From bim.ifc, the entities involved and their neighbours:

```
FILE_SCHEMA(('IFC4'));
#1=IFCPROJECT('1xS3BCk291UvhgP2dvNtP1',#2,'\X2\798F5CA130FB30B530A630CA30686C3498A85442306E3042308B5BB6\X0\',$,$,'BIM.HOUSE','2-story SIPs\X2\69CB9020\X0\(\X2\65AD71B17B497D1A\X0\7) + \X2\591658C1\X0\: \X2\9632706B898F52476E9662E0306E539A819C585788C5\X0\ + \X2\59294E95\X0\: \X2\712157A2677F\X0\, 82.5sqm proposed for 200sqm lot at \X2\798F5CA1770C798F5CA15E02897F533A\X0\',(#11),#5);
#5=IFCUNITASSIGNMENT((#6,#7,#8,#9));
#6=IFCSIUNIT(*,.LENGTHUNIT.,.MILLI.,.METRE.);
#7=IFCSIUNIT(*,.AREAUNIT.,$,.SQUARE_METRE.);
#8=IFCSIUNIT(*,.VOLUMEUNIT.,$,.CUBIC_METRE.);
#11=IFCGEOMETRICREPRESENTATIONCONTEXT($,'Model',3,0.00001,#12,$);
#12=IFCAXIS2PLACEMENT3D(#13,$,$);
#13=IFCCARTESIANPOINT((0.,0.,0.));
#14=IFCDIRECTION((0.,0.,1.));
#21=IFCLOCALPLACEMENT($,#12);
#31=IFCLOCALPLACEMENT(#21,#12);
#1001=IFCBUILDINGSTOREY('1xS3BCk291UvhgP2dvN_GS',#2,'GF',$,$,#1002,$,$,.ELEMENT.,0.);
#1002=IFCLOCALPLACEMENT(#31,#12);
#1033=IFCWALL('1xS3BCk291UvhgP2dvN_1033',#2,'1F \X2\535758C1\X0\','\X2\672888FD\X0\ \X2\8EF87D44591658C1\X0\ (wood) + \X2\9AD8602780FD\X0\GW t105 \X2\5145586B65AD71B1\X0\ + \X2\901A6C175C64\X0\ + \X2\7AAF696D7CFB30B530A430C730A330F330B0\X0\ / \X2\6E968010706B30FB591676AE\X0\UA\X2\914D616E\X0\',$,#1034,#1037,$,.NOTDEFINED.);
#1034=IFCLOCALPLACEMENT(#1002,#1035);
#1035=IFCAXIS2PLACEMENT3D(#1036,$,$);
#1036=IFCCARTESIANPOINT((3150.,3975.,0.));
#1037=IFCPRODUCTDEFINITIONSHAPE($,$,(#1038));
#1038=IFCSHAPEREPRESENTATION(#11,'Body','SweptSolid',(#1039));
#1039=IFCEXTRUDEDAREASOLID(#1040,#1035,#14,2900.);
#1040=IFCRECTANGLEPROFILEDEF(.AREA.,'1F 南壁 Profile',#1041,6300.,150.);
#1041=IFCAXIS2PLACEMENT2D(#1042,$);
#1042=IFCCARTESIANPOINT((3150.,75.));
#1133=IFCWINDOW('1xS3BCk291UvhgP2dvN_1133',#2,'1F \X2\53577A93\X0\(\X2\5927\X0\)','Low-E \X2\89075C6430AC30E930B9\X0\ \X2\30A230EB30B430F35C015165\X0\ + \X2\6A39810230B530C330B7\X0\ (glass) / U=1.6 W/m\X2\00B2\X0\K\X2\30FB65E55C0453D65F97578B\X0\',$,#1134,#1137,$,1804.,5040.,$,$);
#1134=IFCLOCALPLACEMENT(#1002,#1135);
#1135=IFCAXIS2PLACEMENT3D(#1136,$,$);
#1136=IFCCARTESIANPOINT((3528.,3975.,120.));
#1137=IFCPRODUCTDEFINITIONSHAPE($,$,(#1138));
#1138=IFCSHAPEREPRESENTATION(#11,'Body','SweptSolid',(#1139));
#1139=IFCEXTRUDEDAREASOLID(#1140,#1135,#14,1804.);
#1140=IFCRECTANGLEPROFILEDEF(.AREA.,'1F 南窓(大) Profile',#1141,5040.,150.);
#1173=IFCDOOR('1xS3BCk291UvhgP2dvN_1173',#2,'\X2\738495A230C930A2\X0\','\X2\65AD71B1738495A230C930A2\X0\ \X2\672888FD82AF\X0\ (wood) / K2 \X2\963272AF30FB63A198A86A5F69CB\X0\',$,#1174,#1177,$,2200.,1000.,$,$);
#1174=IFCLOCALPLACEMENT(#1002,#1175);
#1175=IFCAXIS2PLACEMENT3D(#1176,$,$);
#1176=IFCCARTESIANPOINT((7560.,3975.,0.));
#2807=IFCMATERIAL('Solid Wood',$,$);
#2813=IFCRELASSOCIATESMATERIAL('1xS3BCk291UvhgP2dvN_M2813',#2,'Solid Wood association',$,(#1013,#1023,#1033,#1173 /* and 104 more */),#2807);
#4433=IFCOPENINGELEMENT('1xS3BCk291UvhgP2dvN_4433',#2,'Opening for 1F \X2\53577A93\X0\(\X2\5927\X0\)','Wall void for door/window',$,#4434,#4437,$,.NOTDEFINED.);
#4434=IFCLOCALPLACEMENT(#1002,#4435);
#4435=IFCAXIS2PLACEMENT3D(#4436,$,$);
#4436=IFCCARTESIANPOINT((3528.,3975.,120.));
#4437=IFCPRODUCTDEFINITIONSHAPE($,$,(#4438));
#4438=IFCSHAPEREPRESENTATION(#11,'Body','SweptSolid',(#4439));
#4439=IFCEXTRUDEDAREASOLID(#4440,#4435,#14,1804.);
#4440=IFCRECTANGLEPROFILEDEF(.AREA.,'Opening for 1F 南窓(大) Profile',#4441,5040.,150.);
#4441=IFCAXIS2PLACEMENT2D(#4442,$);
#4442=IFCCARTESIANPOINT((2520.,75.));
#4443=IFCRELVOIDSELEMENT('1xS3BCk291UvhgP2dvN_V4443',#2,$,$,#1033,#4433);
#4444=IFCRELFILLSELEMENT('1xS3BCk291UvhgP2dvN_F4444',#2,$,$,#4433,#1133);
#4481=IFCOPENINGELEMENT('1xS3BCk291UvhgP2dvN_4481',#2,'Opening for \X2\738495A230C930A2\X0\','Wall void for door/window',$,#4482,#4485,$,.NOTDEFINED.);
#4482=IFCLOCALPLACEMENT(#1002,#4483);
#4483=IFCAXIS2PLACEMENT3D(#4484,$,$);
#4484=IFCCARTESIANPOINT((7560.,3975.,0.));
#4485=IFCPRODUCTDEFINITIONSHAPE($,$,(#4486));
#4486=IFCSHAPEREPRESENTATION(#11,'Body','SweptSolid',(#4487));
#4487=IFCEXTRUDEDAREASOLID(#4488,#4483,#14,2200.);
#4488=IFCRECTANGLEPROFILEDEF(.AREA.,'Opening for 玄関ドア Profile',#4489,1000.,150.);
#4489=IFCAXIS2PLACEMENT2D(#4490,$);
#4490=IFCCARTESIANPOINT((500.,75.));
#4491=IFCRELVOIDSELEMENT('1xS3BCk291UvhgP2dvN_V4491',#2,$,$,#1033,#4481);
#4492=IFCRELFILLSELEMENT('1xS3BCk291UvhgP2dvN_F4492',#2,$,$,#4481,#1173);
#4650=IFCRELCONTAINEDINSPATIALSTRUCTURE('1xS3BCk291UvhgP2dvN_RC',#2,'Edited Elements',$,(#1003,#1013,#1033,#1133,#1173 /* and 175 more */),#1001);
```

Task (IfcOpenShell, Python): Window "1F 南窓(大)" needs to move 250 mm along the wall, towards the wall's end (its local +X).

```python
import ifcopenshell
import ifcopenshell.api.geometry
import ifcopenshell.util.placement
import ifcopenshell.util.unit

model = ifcopenshell.open("bim.ifc")
unit_scale = ifcopenshell.util.unit.calculate_unit_scale(model)

window = model.by_guid("1xS3BCk291UvhgP2dvN_1133")
opening = window.FillsVoids[0].RelatingOpeningElement
wall = opening.VoidsElements[0].RelatingBuildingElement

wall_matrix = ifcopenshell.util.placement.get_local_placement(wall.ObjectPlacement)
shift = wall_matrix[:3, 0] * 0.25 / unit_scale
before = ifcopenshell.util.placement.get_local_placement(window.ObjectPlacement)[:3, 3].copy()

# The window is not placed relative to its opening, so move both.
for product in (opening, window):
    matrix = ifcopenshell.util.placement.get_local_placement(product.ObjectPlacement)
    matrix[:3, 3] += shift
    ifcopenshell.api.geometry.edit_object_placement(model, product=product, matrix=matrix, is_si=False)

after = ifcopenshell.util.placement.get_local_placement(window.ObjectPlacement)[:3, 3]
print("window moved by", (after - before).round(3) + 0.0)

model.write("bim-out.ifc")
```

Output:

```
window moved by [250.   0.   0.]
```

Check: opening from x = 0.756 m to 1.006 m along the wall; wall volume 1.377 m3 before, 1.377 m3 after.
